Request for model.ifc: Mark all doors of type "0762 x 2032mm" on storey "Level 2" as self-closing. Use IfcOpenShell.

First a look at what the model holds.

```python
import ifcopenshell
import ifcopenshell.util.element

model = ifcopenshell.open("model.ifc")
print(model.schema)
storey = next(s for s in model.by_type("IfcBuildingStorey") if s.Name == "Level 2")
doors = [e for e in ifcopenshell.util.element.get_decomposition(storey) if e.is_a("IfcDoor")]
seen = {}
for e in doors:
    element_type = ifcopenshell.util.element.get_type(e)
    key = (element_type.Name if element_type != e and element_type else None, ifcopenshell.util.element.get_pset(e, "Pset_DoorCommon", "SelfClosing"))
    seen[key] = seen.get(key, 0) + 1
for (name, value), count in sorted(seen.items(), key=str):
    print(count, "x", name, "|", value)
```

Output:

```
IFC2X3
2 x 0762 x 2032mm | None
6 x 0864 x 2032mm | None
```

```python
import ifcopenshell
import ifcopenshell.api.pset
import ifcopenshell.util.element

model = ifcopenshell.open("model.ifc")

storey = next(s for s in model.by_type("IfcBuildingStorey") if s.Name == "Level 2")
doors = [e for e in ifcopenshell.util.element.get_decomposition(storey) if e.is_a("IfcDoor")]

count = 0
for e in doors:
    element_type = ifcopenshell.util.element.get_type(e)
    if element_type in (None, e) or element_type.Name != "0762 x 2032mm":
        continue
    # add_pset returns the element's existing set when there is one.
    pset = ifcopenshell.api.pset.add_pset(model, product=e, name="Pset_DoorCommon")
    ifcopenshell.api.pset.edit_pset(model, pset=pset, properties={"SelfClosing": True})
    count += 1

print(count, "doors updated")

model.write("model_updated.ifc")
```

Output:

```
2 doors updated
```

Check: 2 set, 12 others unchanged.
